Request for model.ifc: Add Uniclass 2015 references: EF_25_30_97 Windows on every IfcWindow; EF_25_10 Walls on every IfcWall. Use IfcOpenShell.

First a look at what the model holds.

```python
import ifcopenshell

model = ifcopenshell.open("model.ifc")
print(model.schema)
print("classifications:", [c.Name for c in model.by_type("IfcClassification")])
for ifc_class in ("IfcDoor", "IfcRoof", "IfcStair", "IfcWall", "IfcWindow"):
    print(ifc_class, len(model.by_type(ifc_class)))
```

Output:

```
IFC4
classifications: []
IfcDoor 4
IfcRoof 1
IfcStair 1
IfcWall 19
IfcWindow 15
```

```python
import ifcopenshell
import ifcopenshell.api.classification

model = ifcopenshell.open("model.ifc")

system = ifcopenshell.api.classification.add_classification(model, classification="Uniclass 2015")

codes = {
    "IfcWindow": ("EF_25_30_97", "Windows"),
    "IfcWall": ("EF_25_10", "Walls"),
}
for ifc_class, (code, name) in codes.items():
    products = model.by_type(ifc_class)
    ifcopenshell.api.classification.add_reference(
        model, products=products, classification=system, identification=code, name=name
    )
    print(code, len(products))

model.write("model_rev.ifc")
```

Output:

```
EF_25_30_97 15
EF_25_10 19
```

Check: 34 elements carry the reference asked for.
